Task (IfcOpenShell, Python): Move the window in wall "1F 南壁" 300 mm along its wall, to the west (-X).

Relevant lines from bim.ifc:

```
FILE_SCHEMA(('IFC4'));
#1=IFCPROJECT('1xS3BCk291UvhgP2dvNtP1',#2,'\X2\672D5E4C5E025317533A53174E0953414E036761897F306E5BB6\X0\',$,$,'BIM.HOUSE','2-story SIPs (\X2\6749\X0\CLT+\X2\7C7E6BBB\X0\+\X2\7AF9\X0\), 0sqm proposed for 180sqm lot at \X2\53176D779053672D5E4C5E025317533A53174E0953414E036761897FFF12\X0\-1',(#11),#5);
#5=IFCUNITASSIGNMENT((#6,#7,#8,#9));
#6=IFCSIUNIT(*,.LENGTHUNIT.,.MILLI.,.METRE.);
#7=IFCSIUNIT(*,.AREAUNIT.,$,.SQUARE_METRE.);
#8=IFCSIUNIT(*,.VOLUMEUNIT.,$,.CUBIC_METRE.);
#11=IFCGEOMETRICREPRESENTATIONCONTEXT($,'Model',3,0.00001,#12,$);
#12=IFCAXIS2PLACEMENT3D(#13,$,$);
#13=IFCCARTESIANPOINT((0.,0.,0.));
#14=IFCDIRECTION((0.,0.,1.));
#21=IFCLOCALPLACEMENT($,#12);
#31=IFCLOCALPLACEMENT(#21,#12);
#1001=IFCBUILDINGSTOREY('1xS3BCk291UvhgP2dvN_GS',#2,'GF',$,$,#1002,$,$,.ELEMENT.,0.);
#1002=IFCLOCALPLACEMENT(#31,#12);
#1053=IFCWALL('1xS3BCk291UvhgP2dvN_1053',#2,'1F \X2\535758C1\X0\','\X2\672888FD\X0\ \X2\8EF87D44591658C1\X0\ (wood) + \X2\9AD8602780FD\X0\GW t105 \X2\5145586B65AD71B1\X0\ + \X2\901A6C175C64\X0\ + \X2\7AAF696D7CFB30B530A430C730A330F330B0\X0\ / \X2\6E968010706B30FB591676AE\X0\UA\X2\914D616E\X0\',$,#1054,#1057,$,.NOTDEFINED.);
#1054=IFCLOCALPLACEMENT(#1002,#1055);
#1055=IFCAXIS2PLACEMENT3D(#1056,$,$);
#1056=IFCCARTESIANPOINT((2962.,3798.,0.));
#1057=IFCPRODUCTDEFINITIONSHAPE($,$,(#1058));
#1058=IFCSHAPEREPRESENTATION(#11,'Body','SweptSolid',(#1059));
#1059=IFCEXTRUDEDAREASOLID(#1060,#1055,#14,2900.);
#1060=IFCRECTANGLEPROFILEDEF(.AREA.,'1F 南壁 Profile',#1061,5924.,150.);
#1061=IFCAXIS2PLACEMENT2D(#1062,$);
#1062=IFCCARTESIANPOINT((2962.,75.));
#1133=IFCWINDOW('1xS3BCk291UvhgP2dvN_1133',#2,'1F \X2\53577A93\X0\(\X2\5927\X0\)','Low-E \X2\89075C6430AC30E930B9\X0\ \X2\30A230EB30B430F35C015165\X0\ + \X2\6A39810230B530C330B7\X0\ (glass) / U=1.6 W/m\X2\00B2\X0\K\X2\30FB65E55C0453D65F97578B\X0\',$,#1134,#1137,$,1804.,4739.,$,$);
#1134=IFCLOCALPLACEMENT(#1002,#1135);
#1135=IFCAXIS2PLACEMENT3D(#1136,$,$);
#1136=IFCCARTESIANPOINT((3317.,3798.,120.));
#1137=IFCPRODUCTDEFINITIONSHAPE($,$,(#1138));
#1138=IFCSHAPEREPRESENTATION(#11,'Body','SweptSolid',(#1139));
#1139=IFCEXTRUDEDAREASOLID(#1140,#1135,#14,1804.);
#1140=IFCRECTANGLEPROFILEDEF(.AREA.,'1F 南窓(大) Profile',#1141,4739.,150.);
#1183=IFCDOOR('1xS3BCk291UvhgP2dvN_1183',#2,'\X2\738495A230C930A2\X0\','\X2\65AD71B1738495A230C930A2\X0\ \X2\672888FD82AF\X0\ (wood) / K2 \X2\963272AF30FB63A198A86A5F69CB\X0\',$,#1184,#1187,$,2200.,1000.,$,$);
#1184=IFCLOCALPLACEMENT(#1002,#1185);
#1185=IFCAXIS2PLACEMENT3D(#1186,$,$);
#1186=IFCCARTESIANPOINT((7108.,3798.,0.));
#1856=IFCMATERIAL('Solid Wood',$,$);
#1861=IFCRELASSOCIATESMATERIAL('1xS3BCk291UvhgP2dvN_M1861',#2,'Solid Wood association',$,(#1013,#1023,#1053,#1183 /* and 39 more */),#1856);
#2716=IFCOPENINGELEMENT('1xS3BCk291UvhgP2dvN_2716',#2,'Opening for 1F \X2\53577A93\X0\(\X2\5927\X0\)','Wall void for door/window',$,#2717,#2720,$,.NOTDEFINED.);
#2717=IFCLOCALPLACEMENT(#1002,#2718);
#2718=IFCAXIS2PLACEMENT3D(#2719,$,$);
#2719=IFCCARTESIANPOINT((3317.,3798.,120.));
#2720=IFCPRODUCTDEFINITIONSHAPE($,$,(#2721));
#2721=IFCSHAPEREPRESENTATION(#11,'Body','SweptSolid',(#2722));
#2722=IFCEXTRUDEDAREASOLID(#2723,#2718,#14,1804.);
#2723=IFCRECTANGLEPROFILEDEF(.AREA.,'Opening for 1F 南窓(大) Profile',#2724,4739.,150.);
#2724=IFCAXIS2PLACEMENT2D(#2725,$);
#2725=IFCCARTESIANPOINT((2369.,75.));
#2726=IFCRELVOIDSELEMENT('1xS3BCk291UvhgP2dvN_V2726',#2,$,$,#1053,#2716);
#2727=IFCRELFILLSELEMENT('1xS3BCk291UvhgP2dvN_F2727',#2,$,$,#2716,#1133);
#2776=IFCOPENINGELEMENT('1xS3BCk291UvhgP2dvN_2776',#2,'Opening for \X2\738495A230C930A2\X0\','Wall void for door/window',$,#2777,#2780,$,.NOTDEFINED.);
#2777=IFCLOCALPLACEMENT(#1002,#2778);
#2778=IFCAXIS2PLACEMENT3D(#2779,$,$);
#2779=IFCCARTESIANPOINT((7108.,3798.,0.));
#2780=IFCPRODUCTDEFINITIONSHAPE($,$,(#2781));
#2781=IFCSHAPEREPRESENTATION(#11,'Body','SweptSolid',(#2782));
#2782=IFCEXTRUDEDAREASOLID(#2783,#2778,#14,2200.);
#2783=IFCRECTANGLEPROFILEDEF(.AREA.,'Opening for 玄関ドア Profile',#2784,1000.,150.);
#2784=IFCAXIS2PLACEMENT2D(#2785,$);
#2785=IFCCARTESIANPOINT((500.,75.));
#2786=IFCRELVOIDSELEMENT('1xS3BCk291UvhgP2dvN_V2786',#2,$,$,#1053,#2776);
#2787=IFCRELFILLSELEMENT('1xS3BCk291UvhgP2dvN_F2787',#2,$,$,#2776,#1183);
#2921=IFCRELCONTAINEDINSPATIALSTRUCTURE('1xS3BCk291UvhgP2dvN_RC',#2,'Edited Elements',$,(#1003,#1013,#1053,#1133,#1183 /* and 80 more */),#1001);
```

```python
import ifcopenshell
import ifcopenshell.api.geometry
import ifcopenshell.util.placement
import ifcopenshell.util.unit

model = ifcopenshell.open("bim.ifc")
unit_scale = ifcopenshell.util.unit.calculate_unit_scale(model)

window = model.by_guid("1xS3BCk291UvhgP2dvN_1133")
opening = window.FillsVoids[0].RelatingOpeningElement
wall = opening.VoidsElements[0].RelatingBuildingElement

wall_matrix = ifcopenshell.util.placement.get_local_placement(wall.ObjectPlacement)
shift = wall_matrix[:3, 0] * -0.3 / unit_scale
before = ifcopenshell.util.placement.get_local_placement(window.ObjectPlacement)[:3, 3].copy()

# The window is not placed relative to its opening, so move both.
for product in (opening, window):
    matrix = ifcopenshell.util.placement.get_local_placement(product.ObjectPlacement)
    matrix[:3, 3] += shift
    ifcopenshell.api.geometry.edit_object_placement(model, product=product, matrix=matrix, is_si=False)

after = ifcopenshell.util.placement.get_local_placement(window.ObjectPlacement)[:3, 3]
print("window moved by", (after - before).round(3) + 0.0)

model.write("bim_updated.ifc")
```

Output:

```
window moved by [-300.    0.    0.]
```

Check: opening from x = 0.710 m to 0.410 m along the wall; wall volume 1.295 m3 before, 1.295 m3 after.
